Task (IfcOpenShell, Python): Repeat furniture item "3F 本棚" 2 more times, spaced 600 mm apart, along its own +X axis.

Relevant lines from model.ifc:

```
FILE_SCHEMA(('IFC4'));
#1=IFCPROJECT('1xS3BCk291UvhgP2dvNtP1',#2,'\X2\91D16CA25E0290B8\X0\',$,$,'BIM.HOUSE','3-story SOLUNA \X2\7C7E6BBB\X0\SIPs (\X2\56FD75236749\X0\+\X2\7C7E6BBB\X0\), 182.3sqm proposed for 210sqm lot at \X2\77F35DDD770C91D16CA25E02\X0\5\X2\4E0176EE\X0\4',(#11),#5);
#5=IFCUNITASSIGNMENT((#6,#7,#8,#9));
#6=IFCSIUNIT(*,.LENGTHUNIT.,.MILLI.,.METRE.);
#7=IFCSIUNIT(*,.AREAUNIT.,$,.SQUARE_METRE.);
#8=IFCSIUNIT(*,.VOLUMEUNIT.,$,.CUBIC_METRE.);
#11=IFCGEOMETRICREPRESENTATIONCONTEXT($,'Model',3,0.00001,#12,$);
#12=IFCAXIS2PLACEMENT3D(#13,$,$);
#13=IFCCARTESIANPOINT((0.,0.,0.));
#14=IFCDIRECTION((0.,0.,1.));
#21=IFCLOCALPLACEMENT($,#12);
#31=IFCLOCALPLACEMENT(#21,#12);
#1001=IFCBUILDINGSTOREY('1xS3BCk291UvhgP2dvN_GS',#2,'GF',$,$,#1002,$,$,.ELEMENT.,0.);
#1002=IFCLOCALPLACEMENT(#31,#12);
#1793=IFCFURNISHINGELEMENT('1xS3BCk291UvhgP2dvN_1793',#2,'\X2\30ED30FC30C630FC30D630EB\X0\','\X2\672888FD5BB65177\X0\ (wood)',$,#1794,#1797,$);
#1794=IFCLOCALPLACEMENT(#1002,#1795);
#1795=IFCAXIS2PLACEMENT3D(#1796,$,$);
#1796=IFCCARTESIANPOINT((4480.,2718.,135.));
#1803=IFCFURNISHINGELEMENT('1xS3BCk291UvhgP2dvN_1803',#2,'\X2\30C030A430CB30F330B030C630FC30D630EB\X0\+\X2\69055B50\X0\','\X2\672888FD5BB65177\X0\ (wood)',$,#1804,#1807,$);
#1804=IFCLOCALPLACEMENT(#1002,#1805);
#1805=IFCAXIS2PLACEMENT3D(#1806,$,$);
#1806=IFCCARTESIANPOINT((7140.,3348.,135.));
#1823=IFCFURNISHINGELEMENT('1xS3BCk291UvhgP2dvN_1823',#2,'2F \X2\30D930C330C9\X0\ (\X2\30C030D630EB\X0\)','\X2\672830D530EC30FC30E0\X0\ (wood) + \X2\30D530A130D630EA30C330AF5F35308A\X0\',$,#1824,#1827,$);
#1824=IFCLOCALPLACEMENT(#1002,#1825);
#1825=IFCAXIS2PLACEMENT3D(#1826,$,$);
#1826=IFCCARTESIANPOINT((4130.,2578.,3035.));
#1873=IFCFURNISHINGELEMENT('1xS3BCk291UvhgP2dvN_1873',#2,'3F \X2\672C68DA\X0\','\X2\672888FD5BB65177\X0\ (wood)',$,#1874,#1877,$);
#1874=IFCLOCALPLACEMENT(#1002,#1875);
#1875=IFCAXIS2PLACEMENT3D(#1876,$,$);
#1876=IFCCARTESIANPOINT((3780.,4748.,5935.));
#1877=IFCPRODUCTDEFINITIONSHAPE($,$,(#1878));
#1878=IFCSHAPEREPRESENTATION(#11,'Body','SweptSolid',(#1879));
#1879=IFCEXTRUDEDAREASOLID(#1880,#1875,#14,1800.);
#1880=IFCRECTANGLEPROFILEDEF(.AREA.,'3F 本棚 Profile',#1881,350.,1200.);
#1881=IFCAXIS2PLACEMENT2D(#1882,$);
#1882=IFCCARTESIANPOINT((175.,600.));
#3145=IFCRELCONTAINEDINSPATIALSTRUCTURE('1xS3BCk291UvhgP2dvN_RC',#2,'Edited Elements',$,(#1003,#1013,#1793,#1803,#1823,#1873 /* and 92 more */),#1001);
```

```python
import ifcopenshell
import ifcopenshell.api.geometry
import ifcopenshell.api.root
import ifcopenshell.util.element
import ifcopenshell.util.placement

model = ifcopenshell.open("model.ifc")


def reuse_history(source, copy):
    """copy_class also copies each property set's owner history, people and application; keep the originals."""
    for rel in copy.IsDefinedBy:
        if rel.is_a("IfcRelDefinesByProperties") and (history := rel.RelatingPropertyDefinition.OwnerHistory):
            rel.RelatingPropertyDefinition.OwnerHistory = source.OwnerHistory
            ifcopenshell.util.element.remove_deep2(model, history)


source = model.by_id(1873)
base = ifcopenshell.util.placement.get_local_placement(source.ObjectPlacement)
step = base[:3, 0] * 600.0

for i in range(1, 3):
    copy = ifcopenshell.api.root.copy_class(model, product=source)
    copy.Representation = ifcopenshell.util.element.copy_deep(
        model, source.Representation, exclude=["IfcGeometricRepresentationContext", "IfcRepresentationMap"]
    )
    reuse_history(source, copy)
    matrix = base.copy()
    matrix[:3, 3] += i * step
    print("added at", matrix[:3, 3].round(3) + 0.0)
    ifcopenshell.api.geometry.edit_object_placement(model, product=copy, matrix=matrix, is_si=False)

model.write("model_v2.ifc")
```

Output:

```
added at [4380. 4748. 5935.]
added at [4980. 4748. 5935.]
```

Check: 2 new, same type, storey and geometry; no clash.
